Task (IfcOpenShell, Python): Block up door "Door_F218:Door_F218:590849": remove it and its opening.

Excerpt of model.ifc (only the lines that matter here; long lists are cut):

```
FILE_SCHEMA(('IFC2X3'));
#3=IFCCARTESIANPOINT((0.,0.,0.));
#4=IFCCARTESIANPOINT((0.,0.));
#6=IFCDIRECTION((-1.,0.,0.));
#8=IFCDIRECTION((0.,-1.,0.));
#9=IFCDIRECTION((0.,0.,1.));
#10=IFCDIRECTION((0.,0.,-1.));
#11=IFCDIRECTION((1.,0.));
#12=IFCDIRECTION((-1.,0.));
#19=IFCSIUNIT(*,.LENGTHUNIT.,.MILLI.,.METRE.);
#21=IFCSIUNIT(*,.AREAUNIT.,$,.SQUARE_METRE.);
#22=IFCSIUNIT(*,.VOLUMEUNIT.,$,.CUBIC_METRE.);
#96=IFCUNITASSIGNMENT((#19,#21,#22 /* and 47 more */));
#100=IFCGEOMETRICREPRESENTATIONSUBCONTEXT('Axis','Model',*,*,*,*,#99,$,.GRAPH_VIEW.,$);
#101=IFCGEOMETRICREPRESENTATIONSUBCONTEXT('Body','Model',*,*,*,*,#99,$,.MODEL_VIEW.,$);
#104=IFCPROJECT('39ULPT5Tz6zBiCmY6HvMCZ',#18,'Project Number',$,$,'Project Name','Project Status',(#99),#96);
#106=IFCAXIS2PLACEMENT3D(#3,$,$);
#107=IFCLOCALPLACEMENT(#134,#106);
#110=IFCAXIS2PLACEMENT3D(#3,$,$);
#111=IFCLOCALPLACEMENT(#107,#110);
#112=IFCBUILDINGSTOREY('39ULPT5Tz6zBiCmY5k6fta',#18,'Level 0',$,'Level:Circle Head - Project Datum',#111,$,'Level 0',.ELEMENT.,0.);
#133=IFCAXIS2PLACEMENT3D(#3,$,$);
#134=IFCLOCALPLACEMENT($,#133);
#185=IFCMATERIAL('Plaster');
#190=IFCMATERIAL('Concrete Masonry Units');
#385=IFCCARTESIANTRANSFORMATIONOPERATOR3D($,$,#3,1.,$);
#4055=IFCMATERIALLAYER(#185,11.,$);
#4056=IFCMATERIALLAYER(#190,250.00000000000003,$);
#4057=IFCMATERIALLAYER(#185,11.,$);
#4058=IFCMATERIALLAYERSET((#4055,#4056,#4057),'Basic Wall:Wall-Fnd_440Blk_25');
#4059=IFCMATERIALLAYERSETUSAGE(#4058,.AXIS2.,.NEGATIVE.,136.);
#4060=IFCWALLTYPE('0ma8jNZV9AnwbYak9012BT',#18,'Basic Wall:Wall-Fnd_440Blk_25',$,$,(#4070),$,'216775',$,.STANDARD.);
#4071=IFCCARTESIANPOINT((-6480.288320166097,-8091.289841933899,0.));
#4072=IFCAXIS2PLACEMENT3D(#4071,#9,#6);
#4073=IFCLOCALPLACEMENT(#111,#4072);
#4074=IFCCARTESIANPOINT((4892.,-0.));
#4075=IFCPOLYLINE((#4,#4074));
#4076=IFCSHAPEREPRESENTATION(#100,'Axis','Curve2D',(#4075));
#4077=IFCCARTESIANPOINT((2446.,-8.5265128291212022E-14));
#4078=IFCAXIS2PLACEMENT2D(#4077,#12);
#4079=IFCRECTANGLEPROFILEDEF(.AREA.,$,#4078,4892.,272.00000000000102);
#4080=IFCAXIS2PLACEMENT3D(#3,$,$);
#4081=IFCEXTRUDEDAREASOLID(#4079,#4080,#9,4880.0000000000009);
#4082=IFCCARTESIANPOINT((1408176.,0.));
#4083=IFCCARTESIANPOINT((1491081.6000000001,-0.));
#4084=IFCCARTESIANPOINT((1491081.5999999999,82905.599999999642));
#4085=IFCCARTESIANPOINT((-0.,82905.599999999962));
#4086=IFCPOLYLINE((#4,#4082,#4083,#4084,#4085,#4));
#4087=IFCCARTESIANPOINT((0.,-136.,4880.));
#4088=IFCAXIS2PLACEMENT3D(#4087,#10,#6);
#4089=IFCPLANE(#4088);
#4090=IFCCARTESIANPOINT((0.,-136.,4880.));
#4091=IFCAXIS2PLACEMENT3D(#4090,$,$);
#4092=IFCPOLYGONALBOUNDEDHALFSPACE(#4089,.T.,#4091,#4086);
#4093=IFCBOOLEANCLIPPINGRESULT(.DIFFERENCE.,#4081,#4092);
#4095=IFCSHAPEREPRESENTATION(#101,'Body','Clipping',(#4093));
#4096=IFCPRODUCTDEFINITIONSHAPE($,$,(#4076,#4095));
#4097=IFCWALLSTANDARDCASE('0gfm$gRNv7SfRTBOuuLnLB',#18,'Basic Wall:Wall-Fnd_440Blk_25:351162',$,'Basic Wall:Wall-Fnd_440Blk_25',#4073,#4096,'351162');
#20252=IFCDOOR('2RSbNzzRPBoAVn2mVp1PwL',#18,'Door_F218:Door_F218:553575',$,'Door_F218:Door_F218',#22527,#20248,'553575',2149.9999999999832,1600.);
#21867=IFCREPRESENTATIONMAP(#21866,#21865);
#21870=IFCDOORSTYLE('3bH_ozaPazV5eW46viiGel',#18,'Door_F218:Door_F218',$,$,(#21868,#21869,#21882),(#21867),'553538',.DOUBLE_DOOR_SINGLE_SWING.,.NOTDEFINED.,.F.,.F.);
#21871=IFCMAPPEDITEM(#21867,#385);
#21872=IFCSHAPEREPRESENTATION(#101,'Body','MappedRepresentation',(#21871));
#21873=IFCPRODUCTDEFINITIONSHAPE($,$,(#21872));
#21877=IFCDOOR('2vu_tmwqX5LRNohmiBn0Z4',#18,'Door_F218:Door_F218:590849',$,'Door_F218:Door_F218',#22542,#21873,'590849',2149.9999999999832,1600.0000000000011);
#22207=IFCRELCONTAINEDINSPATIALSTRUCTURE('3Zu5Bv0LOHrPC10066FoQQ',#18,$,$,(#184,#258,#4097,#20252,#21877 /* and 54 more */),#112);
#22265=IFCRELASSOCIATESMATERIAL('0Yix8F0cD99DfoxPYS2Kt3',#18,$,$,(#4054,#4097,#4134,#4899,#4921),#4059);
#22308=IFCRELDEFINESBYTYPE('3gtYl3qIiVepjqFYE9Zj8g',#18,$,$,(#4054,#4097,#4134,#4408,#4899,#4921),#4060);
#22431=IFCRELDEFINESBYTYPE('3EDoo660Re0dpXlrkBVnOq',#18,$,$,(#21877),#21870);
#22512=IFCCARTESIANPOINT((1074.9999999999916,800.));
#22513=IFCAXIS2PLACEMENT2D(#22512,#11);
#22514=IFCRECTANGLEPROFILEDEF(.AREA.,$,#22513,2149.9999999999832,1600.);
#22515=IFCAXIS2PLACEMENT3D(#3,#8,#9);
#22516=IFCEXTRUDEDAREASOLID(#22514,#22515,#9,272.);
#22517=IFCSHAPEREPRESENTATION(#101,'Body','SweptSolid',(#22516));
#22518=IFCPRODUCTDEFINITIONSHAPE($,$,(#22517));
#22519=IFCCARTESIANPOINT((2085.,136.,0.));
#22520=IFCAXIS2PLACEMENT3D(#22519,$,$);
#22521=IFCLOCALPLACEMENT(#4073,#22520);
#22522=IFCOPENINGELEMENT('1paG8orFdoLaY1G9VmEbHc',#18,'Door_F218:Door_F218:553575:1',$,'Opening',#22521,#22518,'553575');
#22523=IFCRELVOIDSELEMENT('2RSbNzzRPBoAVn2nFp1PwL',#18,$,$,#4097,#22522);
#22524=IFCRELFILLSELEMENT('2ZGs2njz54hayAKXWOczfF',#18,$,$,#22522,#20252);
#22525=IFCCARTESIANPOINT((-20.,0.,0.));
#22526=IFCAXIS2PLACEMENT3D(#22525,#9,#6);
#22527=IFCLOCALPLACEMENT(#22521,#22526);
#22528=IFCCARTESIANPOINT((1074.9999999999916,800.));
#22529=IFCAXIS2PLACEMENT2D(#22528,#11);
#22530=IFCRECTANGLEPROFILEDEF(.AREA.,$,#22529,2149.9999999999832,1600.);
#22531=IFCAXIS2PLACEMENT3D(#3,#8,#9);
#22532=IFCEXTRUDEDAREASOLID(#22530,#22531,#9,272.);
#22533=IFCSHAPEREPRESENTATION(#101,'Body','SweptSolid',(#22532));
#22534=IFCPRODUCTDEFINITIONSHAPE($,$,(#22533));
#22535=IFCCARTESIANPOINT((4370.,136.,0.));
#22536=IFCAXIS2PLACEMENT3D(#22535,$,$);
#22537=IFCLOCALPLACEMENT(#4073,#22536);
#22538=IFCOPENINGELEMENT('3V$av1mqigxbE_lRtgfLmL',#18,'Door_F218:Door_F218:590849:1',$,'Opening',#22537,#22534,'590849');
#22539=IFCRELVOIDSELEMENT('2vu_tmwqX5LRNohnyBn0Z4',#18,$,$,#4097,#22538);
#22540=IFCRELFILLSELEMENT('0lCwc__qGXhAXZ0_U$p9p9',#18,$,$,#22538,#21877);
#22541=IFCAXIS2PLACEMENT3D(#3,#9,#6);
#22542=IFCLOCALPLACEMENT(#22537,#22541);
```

```python
import ifcopenshell
import ifcopenshell.api.feature
import ifcopenshell.api.root
import ifcopenshell.geom
import ifcopenshell.util.shape

model = ifcopenshell.open("model.ifc")
settings = ifcopenshell.geom.settings()


def volume(element):
    """Net volume in cubic metres, openings subtracted."""
    shape = ifcopenshell.geom.create_shape(settings, element)
    return ifcopenshell.util.shape.get_volume(shape.geometry)


door = model.by_guid("2vu_tmwqX5LRNohmiBn0Z4")
opening = door.FillsVoids[0].RelatingOpeningElement
wall = opening.VoidsElements[0].RelatingBuildingElement
before = volume(wall)

ifcopenshell.api.root.remove_product(model, product=door)
ifcopenshell.api.feature.remove_feature(model, feature=opening)

after = volume(wall)

print(f"wall volume {before:.3f} -> {after:.3f} m3")

model.write("model_rev.ifc")
```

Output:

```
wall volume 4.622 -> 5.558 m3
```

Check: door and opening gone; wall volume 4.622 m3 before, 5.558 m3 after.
